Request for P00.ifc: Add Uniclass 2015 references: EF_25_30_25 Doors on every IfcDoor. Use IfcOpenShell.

First a look at what the model holds.

```python
import ifcopenshell

model = ifcopenshell.open("P00.ifc")
print(model.schema)
print("classifications:", [c.Name for c in model.by_type("IfcClassification")])
for ifc_class in ("IfcDoor", "IfcRoof", "IfcStair", "IfcWall", "IfcWindow"):
    print(ifc_class, len(model.by_type(ifc_class)))
```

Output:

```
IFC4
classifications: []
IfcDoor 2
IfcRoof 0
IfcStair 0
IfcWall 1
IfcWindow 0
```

```python
import ifcopenshell
import ifcopenshell.api.classification

model = ifcopenshell.open("P00.ifc")

system = ifcopenshell.api.classification.add_classification(model, classification="Uniclass 2015")

codes = {
    "IfcDoor": ("EF_25_30_25", "Doors"),
}
for ifc_class, (code, name) in codes.items():
    products = model.by_type(ifc_class)
    ifcopenshell.api.classification.add_reference(
        model, products=products, classification=system, identification=code, name=name
    )
    print(code, len(products))

model.write("P00_rev.ifc")
```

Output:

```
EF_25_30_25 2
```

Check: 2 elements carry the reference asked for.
